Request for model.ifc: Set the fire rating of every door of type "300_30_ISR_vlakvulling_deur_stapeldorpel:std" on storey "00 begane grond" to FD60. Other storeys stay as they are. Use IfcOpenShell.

First a look at what the model holds.

```python
import ifcopenshell
import ifcopenshell.util.element

model = ifcopenshell.open("model.ifc")
print(model.schema)
storey = next(s for s in model.by_type("IfcBuildingStorey") if s.Name == "00 begane grond")
doors = [e for e in ifcopenshell.util.element.get_decomposition(storey) if e.is_a("IfcDoor")]
seen = {}
for e in doors:
    element_type = ifcopenshell.util.element.get_type(e)
    key = (element_type.Name if element_type != e and element_type else None, ifcopenshell.util.element.get_pset(e, "Pset_DoorCommon", "FireRating"))
    seen[key] = seen.get(key, 0) + 1
for (name, value), count in sorted(seen.items(), key=str):
    print(count, "x", name, "|", value)
```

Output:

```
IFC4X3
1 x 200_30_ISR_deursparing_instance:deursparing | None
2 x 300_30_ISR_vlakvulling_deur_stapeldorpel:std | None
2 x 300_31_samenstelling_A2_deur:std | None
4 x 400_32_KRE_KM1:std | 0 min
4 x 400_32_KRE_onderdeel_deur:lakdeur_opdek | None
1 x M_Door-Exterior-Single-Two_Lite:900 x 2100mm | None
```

```python
import ifcopenshell
import ifcopenshell.api.pset
import ifcopenshell.util.element

model = ifcopenshell.open("model.ifc")

storey = next(s for s in model.by_type("IfcBuildingStorey") if s.Name == "00 begane grond")
doors = [e for e in ifcopenshell.util.element.get_decomposition(storey) if e.is_a("IfcDoor")]

count = 0
for e in doors:
    element_type = ifcopenshell.util.element.get_type(e)
    if element_type in (None, e) or element_type.Name != "300_30_ISR_vlakvulling_deur_stapeldorpel:std":
        continue
    # add_pset returns the element's existing set when there is one.
    pset = ifcopenshell.api.pset.add_pset(model, product=e, name="Pset_DoorCommon")
    ifcopenshell.api.pset.edit_pset(model, pset=pset, properties={"FireRating": "FD60"})
    count += 1

print(count, "doors updated")

model.write("model_rev.ifc")
```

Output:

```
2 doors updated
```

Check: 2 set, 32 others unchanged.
